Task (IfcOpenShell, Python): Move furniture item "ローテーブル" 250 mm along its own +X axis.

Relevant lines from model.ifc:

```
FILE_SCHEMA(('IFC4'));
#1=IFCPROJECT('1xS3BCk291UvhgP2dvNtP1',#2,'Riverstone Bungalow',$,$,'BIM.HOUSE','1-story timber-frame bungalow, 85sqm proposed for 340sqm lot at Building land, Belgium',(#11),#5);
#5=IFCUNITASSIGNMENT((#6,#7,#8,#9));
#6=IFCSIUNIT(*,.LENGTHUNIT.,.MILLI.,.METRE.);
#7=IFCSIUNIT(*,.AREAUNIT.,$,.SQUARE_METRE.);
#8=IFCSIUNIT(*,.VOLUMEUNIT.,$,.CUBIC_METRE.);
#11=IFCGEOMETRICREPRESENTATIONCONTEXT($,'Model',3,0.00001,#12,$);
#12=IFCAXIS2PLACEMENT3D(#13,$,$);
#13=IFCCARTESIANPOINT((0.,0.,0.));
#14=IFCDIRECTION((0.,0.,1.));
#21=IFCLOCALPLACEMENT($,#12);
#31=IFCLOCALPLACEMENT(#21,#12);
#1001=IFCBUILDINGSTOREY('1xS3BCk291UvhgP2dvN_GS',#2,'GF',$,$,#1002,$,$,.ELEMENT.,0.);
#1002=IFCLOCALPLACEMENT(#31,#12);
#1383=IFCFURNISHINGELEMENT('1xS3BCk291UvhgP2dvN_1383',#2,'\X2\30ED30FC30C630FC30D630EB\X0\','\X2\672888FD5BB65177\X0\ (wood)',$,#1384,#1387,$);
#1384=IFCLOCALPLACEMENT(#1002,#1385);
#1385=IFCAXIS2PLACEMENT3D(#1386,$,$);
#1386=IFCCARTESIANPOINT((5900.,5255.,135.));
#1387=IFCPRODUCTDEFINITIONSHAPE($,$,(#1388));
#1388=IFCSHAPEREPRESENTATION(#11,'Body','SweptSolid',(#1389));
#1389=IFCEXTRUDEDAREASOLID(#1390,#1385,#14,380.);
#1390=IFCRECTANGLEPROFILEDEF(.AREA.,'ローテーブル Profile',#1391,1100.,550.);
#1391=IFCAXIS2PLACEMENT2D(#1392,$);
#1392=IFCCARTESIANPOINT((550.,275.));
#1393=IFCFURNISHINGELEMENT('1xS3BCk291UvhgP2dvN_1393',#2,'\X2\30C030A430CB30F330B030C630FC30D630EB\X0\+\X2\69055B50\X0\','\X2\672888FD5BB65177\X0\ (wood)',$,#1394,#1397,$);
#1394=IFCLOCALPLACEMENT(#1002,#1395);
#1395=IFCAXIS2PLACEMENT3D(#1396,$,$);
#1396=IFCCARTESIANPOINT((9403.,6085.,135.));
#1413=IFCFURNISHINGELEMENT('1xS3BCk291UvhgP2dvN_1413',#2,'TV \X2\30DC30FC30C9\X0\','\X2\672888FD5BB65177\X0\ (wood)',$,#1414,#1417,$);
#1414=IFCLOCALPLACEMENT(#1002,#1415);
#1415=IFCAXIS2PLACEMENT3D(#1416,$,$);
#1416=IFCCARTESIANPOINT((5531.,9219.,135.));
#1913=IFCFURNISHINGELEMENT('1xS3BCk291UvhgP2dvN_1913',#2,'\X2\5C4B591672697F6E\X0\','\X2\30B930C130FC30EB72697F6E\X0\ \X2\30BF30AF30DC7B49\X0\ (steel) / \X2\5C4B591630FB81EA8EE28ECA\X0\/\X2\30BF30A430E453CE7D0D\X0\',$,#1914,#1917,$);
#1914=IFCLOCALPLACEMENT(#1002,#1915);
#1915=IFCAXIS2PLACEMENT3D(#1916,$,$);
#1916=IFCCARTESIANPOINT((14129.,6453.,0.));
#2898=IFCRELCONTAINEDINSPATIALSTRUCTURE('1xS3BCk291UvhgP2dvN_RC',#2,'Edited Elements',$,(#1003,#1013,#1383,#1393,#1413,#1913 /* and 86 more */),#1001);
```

```python
import ifcopenshell
import ifcopenshell.api.geometry
import ifcopenshell.util.placement
import ifcopenshell.util.unit

model = ifcopenshell.open("model.ifc")
unit_scale = ifcopenshell.util.unit.calculate_unit_scale(model)

item = model.by_id(1383)
matrix = ifcopenshell.util.placement.get_local_placement(item.ObjectPlacement)
matrix[:3, 3] += matrix[:3, 0] * 0.25 / unit_scale
ifcopenshell.api.geometry.edit_object_placement(model, product=item, matrix=matrix, is_si=False)

print(ifcopenshell.util.placement.get_local_placement(item.ObjectPlacement).round(3) + 0.0)

model.write("model_edited.ifc")
```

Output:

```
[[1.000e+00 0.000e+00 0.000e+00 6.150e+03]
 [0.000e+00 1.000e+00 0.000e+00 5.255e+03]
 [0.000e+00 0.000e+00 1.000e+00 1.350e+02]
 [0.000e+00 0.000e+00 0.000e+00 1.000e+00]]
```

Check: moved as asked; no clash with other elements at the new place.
